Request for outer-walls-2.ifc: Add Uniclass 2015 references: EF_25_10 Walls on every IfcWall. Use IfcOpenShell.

First a look at what the model holds.

```python
import ifcopenshell

model = ifcopenshell.open("outer-walls-2.ifc")
print(model.schema)
print("classifications:", [c.Name for c in model.by_type("IfcClassification")])
for ifc_class in ("IfcDoor", "IfcRoof", "IfcStair", "IfcWall", "IfcWindow"):
    print(ifc_class, len(model.by_type(ifc_class)))
```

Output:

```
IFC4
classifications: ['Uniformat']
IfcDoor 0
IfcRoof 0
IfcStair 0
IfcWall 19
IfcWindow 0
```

```python
import ifcopenshell
import ifcopenshell.api.classification

model = ifcopenshell.open("outer-walls-2.ifc")

system = ifcopenshell.api.classification.add_classification(model, classification="Uniclass 2015")

codes = {
    "IfcWall": ("EF_25_10", "Walls"),
}
for ifc_class, (code, name) in codes.items():
    products = model.by_type(ifc_class)
    ifcopenshell.api.classification.add_reference(
        model, products=products, classification=system, identification=code, name=name
    )
    print(code, len(products))

model.write("outer-walls-2_updated.ifc")
```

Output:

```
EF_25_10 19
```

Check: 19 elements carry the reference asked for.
